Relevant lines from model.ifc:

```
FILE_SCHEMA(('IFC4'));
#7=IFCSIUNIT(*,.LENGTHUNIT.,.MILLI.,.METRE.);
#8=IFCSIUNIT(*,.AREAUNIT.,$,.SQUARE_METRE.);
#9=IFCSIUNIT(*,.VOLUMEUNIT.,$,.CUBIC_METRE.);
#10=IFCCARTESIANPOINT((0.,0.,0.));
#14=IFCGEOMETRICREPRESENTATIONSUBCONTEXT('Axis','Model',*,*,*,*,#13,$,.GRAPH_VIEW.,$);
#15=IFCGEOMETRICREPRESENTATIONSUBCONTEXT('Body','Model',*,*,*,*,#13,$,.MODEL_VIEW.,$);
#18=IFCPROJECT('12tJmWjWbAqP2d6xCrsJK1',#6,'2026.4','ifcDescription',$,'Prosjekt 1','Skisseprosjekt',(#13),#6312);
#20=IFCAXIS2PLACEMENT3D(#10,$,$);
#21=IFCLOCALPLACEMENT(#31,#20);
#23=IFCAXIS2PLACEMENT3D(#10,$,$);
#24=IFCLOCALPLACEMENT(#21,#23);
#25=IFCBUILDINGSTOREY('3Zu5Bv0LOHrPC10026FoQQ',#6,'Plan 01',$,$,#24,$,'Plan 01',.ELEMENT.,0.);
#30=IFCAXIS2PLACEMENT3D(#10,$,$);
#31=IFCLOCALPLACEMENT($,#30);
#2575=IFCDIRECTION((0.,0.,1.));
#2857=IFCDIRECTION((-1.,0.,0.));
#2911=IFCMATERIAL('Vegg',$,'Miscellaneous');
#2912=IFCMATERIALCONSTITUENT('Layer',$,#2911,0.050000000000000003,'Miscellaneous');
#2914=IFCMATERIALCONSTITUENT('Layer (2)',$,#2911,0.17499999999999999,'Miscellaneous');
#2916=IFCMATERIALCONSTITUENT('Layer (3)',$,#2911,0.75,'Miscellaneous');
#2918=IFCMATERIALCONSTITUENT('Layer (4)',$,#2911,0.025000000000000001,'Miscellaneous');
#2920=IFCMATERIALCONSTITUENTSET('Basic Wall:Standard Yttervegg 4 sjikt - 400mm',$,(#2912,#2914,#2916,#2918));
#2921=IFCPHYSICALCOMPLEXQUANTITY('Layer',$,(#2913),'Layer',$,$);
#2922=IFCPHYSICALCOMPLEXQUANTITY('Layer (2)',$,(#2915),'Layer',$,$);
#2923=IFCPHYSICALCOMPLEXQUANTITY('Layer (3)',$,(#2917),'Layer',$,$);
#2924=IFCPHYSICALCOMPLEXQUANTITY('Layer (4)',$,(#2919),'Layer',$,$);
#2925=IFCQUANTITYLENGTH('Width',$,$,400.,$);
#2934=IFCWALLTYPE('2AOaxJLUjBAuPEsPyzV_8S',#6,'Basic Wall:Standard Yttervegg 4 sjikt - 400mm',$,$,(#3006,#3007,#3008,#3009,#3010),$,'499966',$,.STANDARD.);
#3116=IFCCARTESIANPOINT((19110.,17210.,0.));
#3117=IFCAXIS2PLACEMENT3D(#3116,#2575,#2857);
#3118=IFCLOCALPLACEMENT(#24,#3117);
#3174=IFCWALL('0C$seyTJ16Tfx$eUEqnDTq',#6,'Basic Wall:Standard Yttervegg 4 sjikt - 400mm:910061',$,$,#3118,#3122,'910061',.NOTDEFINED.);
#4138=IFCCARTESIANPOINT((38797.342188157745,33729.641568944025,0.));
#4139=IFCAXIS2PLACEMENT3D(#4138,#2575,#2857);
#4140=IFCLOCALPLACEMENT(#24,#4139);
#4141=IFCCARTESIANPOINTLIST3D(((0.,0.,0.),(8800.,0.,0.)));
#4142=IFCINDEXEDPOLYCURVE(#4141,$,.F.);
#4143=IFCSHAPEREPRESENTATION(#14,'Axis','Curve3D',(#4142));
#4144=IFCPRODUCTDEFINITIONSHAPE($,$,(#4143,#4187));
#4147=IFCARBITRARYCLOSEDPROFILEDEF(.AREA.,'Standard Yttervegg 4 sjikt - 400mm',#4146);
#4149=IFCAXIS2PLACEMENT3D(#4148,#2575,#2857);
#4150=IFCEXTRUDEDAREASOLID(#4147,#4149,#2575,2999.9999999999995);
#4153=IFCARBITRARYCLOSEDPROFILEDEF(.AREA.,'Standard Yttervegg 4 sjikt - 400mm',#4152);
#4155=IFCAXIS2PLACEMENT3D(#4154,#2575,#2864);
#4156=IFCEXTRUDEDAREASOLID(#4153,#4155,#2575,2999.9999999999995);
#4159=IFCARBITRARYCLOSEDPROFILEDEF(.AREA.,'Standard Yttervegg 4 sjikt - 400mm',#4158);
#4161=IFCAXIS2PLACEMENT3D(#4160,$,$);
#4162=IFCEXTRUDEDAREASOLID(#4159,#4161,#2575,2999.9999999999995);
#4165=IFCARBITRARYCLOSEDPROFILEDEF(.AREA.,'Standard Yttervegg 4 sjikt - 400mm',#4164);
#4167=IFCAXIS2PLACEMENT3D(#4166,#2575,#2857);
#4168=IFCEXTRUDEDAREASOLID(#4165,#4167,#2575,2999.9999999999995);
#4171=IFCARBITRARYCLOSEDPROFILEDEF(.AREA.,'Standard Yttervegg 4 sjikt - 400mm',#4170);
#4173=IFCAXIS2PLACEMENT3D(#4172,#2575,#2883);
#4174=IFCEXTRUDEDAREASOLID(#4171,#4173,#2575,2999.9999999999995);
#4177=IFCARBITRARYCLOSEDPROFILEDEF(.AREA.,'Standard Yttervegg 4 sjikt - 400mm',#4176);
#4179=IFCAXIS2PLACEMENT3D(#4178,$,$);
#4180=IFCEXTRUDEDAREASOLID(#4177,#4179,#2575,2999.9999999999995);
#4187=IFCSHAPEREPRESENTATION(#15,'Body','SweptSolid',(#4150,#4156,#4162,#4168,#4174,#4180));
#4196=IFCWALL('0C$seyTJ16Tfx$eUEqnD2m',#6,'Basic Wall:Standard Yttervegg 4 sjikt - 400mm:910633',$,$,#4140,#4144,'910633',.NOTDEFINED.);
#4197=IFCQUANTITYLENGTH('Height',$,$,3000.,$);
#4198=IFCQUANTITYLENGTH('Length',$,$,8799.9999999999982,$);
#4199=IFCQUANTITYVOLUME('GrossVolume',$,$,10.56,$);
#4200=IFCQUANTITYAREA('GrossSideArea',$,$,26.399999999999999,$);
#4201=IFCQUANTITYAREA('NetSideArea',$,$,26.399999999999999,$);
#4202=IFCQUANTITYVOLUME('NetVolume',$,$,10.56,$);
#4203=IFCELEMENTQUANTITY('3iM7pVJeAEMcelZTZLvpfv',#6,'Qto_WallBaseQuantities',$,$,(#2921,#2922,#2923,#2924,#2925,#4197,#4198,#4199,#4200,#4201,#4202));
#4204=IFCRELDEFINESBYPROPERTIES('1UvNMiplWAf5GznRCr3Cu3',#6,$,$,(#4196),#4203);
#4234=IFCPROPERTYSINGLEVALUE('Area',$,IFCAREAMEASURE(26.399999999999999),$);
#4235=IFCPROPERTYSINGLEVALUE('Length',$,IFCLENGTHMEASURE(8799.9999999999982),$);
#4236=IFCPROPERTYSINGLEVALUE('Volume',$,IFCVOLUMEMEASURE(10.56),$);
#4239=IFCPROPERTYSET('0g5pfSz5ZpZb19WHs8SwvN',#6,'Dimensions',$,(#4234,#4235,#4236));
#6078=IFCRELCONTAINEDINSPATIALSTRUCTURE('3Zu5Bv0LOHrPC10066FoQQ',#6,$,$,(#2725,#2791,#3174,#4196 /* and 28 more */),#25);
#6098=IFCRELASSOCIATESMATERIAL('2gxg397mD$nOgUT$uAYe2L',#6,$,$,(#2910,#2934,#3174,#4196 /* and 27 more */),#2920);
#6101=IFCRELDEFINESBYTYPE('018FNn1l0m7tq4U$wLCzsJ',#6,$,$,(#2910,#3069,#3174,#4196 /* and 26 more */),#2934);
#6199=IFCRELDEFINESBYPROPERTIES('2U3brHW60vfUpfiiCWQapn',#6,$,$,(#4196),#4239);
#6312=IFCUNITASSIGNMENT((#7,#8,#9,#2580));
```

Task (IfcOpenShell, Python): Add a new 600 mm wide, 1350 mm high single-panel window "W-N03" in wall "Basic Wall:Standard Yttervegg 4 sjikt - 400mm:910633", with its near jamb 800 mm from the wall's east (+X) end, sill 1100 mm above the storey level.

```python
import numpy as np
import ifcopenshell
import ifcopenshell.api.feature
import ifcopenshell.api.geometry
import ifcopenshell.api.pset
import ifcopenshell.api.root
import ifcopenshell.api.spatial
import ifcopenshell.geom
import ifcopenshell.util.element
import ifcopenshell.util.placement
import ifcopenshell.util.representation
import ifcopenshell.util.shape
import ifcopenshell.util.unit

model = ifcopenshell.open("model.ifc")
unit_scale = ifcopenshell.util.unit.calculate_unit_scale(model)
area_scale = ifcopenshell.util.unit.calculate_unit_scale(model, "AREAUNIT")
volume_scale = ifcopenshell.util.unit.calculate_unit_scale(model, "VOLUMEUNIT")
settings = ifcopenshell.geom.settings()


def volume(element):
    """Net volume in cubic metres, openings subtracted."""
    shape = ifcopenshell.geom.create_shape(settings, element)
    return ifcopenshell.util.shape.get_volume(shape.geometry)


wall = model.by_guid("0C$seyTJ16Tfx$eUEqnD2m")
storey = ifcopenshell.util.element.get_container(wall, ifc_class="IfcBuildingStorey")
context = ifcopenshell.util.representation.get_context(model, "Model", "Body", "MODEL_VIEW")
before = volume(wall)

width, height, from_end, sill = 0.6, 1.35, 0.8, 1.1  # metres

# The wall runs along its own X axis, and the end named is its -X end.
wall_shape = ifcopenshell.geom.create_shape(settings, wall)
x, y, z = ifcopenshell.util.shape.get_vertices(wall_shape.geometry).T
start = x.min() + from_end
face, thickness = float(y.min()), float(y.max() - y.min())
wall_matrix = ifcopenshell.util.placement.get_local_placement(wall.ObjectPlacement)
level = ifcopenshell.util.placement.get_local_placement(storey.ObjectPlacement)[2, 3]


def in_wall(x, y):
    """Placement at x, y metres in the wall's axes, at sill height."""
    matrix = wall_matrix.copy()
    matrix[:, 3] = wall_matrix @ np.array([x / unit_scale, y / unit_scale, 0.0, 1.0])
    matrix[2, 3] = level + sill / unit_scale
    return matrix


# Opening: a box that overshoots both wall faces by 50 mm.
opening = ifcopenshell.api.root.create_entity(model, ifc_class="IfcOpeningElement", predefined_type="OPENING")
box = ifcopenshell.api.geometry.add_wall_representation(
    model, context=context, length=width, height=height, thickness=thickness + 0.1
)
ifcopenshell.api.geometry.assign_representation(model, product=opening, representation=box)
ifcopenshell.api.geometry.edit_object_placement(model, product=opening, matrix=in_wall(start, face - 0.05), is_si=False)
ifcopenshell.api.feature.add_feature(model, feature=opening, element=wall)

window = ifcopenshell.api.root.create_entity(model, ifc_class="IfcWindow", name="W-N03", predefined_type="WINDOW")
window.OverallWidth, window.OverallHeight = width / unit_scale, height / unit_scale
window.PartitioningType = "SINGLE_PANEL"
body = ifcopenshell.api.geometry.add_window_representation(
    model,
    context=context,
    overall_width=window.OverallWidth,
    overall_height=window.OverallHeight,
    partition_type="SINGLE_PANEL",
)
ifcopenshell.api.geometry.assign_representation(model, product=window, representation=body)
ifcopenshell.api.spatial.assign_container(model, products=[window], relating_structure=storey)
ifcopenshell.api.feature.add_filling(model, opening=opening, element=window)

# Centre the window in the wall's thickness.
ifcopenshell.api.geometry.edit_object_placement(model, product=window, matrix=in_wall(start, face), is_si=False)
window_shape = ifcopenshell.geom.create_shape(settings, window)
depth = ifcopenshell.util.shape.get_vertices(window_shape.geometry)[:, 1]
offset = face + thickness / 2 - (depth.min() + depth.max()) / 2
ifcopenshell.api.geometry.edit_object_placement(model, product=window, matrix=in_wall(start, offset), is_si=False)

after = volume(wall)

# Update the wall's stored quantities.
qto = model.by_id(ifcopenshell.util.element.get_pset(wall, "Qto_WallBaseQuantities", should_inherit=False)["id"])
ifcopenshell.api.pset.edit_qto(model, qto=qto, properties={
    "NetSideArea": after / thickness / area_scale,
    "NetVolume": after / volume_scale,
})
pset = model.by_id(ifcopenshell.util.element.get_pset(wall, "Dimensions", should_inherit=False)["id"])
ifcopenshell.api.pset.edit_pset(model, pset=pset, properties={
    "Area": model.create_entity("IfcAreaMeasure", after / thickness / area_scale),
    "Volume": model.create_entity("IfcVolumeMeasure", after / volume_scale),
})

print(f"wall volume {before:.3f} -> {after:.3f} m3")

model.write("model_rev.ifc")
```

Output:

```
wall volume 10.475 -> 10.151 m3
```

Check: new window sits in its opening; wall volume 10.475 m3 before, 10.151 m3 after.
